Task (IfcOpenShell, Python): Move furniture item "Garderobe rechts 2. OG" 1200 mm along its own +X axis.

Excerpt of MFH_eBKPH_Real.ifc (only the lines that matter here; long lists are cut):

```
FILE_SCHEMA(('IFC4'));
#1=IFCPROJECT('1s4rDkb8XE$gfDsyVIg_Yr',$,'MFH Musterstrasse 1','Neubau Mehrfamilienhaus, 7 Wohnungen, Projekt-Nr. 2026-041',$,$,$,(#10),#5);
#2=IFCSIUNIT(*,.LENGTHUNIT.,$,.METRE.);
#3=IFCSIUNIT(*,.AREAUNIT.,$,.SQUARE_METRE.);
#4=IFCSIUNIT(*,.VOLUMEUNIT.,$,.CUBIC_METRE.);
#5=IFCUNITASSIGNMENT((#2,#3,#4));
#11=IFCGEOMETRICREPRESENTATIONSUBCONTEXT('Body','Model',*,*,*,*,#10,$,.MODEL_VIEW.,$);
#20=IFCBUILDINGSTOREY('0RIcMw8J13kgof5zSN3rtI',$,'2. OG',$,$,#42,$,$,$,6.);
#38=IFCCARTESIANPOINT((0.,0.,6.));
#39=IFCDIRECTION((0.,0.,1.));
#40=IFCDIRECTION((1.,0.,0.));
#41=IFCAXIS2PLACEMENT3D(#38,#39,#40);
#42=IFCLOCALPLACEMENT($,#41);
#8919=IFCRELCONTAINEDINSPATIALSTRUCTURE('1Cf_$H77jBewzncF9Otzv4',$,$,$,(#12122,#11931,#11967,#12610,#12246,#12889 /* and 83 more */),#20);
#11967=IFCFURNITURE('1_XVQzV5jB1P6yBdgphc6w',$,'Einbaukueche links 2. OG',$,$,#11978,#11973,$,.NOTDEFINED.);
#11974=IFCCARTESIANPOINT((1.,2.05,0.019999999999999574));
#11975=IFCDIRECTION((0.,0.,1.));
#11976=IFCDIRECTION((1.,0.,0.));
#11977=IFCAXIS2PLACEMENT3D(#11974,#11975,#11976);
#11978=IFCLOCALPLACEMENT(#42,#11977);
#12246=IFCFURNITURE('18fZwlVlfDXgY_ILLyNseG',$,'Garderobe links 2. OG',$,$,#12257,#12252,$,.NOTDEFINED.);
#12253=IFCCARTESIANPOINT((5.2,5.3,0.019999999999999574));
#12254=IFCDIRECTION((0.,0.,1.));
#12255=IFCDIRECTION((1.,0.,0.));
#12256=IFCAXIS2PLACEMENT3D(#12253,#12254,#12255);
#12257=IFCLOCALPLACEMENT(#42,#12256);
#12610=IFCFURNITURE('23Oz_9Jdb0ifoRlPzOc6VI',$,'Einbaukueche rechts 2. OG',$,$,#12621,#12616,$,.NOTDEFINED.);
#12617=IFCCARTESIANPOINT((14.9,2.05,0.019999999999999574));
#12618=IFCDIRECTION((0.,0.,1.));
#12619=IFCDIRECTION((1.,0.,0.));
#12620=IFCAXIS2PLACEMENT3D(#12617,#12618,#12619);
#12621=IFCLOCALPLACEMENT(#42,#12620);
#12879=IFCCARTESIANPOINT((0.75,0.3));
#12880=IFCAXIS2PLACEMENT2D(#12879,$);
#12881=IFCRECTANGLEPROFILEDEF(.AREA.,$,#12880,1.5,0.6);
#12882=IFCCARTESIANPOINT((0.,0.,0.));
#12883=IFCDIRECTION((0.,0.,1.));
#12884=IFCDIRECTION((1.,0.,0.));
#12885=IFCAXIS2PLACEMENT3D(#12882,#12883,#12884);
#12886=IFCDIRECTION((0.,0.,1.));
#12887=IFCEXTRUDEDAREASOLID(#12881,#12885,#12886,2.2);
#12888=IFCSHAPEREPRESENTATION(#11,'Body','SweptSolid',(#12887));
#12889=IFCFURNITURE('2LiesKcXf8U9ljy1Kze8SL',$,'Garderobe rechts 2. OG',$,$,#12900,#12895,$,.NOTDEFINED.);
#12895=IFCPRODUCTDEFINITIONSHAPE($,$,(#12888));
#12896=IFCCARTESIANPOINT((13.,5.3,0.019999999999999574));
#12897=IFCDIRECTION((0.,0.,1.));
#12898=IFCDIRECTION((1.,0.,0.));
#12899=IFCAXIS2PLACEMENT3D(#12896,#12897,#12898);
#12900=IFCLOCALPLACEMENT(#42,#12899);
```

```python
import ifcopenshell
import ifcopenshell.api.geometry
import ifcopenshell.util.placement

model = ifcopenshell.open("MFH_eBKPH_Real.ifc")

item = model.by_guid("2LiesKcXf8U9ljy1Kze8SL")
matrix = ifcopenshell.util.placement.get_local_placement(item.ObjectPlacement)
matrix[:3, 3] += matrix[:3, 0] * 1.2
ifcopenshell.api.geometry.edit_object_placement(model, product=item, matrix=matrix, is_si=False)

print(ifcopenshell.util.placement.get_local_placement(item.ObjectPlacement).round(3) + 0.0)

model.write("MFH_eBKPH_Real_updated.ifc")
```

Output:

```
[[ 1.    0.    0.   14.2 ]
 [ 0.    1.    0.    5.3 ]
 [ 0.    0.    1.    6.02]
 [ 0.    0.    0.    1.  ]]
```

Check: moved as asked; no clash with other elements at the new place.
